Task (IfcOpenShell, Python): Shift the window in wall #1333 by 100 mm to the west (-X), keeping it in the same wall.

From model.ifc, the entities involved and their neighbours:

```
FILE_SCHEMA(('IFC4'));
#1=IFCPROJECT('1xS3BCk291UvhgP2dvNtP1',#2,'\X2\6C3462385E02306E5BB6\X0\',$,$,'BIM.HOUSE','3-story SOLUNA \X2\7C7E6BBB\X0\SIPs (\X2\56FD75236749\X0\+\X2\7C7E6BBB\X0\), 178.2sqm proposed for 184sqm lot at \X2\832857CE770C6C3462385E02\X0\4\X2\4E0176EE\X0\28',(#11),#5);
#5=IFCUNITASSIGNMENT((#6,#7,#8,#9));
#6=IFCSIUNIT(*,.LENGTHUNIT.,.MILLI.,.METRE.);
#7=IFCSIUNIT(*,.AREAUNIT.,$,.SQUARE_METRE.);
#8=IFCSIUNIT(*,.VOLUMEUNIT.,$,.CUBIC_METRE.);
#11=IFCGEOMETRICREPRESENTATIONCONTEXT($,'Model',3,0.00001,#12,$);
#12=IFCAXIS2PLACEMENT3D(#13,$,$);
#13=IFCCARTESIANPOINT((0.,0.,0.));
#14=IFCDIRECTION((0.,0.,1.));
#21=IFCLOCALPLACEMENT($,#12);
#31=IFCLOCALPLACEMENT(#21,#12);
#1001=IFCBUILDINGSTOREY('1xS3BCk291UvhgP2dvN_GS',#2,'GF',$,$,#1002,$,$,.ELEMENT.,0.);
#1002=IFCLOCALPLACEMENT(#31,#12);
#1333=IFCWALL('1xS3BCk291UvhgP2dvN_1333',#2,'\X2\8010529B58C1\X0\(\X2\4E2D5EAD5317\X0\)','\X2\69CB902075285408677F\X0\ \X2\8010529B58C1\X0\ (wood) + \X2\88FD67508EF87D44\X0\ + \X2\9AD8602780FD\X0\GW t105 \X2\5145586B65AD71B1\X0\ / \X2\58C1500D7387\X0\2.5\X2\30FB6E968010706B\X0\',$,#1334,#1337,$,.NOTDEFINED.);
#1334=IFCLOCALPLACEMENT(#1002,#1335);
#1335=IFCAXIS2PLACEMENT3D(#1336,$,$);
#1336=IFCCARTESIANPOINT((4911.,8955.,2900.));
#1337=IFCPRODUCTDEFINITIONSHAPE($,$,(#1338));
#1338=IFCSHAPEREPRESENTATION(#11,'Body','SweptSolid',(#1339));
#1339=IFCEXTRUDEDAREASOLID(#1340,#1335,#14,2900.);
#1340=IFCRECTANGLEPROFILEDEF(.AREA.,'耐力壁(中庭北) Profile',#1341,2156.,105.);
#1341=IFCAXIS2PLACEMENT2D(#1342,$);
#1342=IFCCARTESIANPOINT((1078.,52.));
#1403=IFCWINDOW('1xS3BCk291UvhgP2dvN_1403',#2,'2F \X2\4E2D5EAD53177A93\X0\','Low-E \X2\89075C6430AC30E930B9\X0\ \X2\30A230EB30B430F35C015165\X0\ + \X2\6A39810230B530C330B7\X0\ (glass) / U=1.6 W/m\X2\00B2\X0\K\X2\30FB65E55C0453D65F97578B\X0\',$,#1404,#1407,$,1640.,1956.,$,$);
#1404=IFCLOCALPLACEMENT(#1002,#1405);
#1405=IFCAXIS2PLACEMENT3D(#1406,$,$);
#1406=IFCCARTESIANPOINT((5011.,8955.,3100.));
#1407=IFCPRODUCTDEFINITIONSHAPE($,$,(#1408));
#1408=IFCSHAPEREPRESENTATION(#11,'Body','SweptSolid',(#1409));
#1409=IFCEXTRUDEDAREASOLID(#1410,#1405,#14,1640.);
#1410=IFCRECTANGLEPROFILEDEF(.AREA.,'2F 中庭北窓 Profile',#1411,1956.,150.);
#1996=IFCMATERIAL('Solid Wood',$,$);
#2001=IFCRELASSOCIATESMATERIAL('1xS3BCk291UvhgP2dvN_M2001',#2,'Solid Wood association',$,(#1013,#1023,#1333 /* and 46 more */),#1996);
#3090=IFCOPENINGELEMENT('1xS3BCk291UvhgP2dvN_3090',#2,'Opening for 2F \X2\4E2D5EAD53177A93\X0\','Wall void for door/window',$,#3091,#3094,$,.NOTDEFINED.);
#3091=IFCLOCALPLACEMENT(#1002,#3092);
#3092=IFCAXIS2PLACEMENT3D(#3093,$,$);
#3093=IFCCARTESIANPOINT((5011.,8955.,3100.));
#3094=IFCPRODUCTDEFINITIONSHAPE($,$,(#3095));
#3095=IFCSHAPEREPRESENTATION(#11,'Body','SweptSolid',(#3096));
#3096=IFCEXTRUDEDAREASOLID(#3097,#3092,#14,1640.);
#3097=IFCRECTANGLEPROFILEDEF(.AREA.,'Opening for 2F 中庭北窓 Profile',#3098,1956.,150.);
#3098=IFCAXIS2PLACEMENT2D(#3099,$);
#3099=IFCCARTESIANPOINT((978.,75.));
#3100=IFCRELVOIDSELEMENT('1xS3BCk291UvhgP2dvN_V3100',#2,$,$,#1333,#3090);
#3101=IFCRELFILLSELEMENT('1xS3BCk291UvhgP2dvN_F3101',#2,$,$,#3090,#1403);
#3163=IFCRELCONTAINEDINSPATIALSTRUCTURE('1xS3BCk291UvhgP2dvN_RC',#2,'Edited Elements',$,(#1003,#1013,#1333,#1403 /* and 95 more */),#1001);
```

```python
import ifcopenshell
import ifcopenshell.api.geometry
import ifcopenshell.util.placement
import ifcopenshell.util.unit

model = ifcopenshell.open("model.ifc")
unit_scale = ifcopenshell.util.unit.calculate_unit_scale(model)

window = model.by_id(1403)
opening = window.FillsVoids[0].RelatingOpeningElement
wall = opening.VoidsElements[0].RelatingBuildingElement

wall_matrix = ifcopenshell.util.placement.get_local_placement(wall.ObjectPlacement)
shift = wall_matrix[:3, 0] * -0.1 / unit_scale
before = ifcopenshell.util.placement.get_local_placement(window.ObjectPlacement)[:3, 3].copy()

# The window is not placed relative to its opening, so move both.
for product in (opening, window):
    matrix = ifcopenshell.util.placement.get_local_placement(product.ObjectPlacement)
    matrix[:3, 3] += shift
    ifcopenshell.api.geometry.edit_object_placement(model, product=product, matrix=matrix, is_si=False)

after = ifcopenshell.util.placement.get_local_placement(window.ObjectPlacement)[:3, 3]
print("window moved by", (after - before).round(3) + 0.0)

model.write("model_v2.ifc")
```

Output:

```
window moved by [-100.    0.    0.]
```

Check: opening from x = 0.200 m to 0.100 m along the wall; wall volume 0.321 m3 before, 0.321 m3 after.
